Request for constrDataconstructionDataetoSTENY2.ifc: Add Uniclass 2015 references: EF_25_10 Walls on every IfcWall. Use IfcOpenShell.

First a look at what the model holds.

```python
import ifcopenshell

model = ifcopenshell.open("constrDataconstructionDataetoSTENY2.ifc")
print(model.schema)
print("classifications:", [c.Name for c in model.by_type("IfcClassification")])
for ifc_class in ("IfcDoor", "IfcRoof", "IfcStair", "IfcWall", "IfcWindow"):
    print(ifc_class, len(model.by_type(ifc_class)))
```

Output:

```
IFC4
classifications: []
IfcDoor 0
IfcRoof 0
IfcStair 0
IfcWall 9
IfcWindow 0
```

```python
import ifcopenshell
import ifcopenshell.api.classification

model = ifcopenshell.open("constrDataconstructionDataetoSTENY2.ifc")

system = ifcopenshell.api.classification.add_classification(model, classification="Uniclass 2015")

codes = {
    "IfcWall": ("EF_25_10", "Walls"),
}
for ifc_class, (code, name) in codes.items():
    products = model.by_type(ifc_class)
    ifcopenshell.api.classification.add_reference(
        model, products=products, classification=system, identification=code, name=name
    )
    print(code, len(products))

model.write("constrDataconstructionDataetoSTENY2_updated.ifc")
```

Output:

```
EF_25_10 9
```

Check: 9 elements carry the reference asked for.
